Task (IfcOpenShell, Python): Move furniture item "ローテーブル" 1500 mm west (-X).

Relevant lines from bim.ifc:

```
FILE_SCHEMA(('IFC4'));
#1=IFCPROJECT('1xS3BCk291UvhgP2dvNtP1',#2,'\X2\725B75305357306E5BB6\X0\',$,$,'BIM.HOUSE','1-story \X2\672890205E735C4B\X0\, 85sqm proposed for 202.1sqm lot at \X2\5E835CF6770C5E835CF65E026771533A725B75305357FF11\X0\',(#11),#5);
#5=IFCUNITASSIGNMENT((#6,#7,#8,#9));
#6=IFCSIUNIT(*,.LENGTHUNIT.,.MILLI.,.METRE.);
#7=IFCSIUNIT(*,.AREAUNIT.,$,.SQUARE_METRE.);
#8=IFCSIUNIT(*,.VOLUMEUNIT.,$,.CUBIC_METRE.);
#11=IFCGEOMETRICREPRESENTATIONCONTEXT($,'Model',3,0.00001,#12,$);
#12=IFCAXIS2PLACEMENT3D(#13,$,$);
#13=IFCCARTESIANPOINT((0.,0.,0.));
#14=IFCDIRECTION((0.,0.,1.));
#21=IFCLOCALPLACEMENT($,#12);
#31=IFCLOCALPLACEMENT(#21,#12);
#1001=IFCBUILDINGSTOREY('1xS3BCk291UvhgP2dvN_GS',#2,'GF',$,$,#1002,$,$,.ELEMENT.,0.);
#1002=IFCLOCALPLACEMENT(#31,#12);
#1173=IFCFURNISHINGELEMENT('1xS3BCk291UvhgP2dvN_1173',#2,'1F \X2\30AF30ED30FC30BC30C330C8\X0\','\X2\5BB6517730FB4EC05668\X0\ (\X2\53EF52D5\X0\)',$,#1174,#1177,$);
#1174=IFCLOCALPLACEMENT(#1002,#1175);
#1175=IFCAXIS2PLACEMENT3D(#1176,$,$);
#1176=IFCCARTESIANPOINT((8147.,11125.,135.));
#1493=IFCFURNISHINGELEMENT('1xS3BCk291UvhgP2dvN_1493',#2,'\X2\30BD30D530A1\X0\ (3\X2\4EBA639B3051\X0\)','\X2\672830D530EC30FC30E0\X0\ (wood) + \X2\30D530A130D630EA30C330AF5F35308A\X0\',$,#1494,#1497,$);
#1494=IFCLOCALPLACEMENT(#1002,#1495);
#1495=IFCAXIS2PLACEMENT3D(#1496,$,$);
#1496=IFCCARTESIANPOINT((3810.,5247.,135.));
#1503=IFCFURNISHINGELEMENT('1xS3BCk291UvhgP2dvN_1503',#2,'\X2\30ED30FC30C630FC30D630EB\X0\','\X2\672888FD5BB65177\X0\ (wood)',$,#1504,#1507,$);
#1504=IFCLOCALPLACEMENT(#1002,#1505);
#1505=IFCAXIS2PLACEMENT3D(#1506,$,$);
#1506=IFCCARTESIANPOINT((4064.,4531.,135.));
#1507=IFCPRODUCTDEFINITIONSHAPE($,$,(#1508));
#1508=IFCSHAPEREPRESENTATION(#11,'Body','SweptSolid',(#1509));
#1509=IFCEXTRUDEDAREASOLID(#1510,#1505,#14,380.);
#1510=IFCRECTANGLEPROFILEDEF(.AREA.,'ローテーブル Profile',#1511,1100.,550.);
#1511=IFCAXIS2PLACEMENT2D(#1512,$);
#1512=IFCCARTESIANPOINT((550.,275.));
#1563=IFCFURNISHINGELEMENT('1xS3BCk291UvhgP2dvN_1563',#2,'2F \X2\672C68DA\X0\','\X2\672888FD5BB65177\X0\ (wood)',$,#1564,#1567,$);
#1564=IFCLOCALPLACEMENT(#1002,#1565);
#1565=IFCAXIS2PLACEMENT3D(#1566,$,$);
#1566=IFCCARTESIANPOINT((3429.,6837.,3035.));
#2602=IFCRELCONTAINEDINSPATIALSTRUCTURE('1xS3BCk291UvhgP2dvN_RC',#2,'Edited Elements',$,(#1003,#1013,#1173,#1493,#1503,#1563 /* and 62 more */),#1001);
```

```python
import ifcopenshell
import ifcopenshell.api.geometry
import ifcopenshell.util.placement
import ifcopenshell.util.unit

model = ifcopenshell.open("bim.ifc")
unit_scale = ifcopenshell.util.unit.calculate_unit_scale(model)

item = model.by_guid("1xS3BCk291UvhgP2dvN_1503")
matrix = ifcopenshell.util.placement.get_local_placement(item.ObjectPlacement)
matrix[0, 3] -= 1.5 / unit_scale
ifcopenshell.api.geometry.edit_object_placement(model, product=item, matrix=matrix, is_si=False)

print(ifcopenshell.util.placement.get_local_placement(item.ObjectPlacement).round(3) + 0.0)

model.write("bim_v2.ifc")
```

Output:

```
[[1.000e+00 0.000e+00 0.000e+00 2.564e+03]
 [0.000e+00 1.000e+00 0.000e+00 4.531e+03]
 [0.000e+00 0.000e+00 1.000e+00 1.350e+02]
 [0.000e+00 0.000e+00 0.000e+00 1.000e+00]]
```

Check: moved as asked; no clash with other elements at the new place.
